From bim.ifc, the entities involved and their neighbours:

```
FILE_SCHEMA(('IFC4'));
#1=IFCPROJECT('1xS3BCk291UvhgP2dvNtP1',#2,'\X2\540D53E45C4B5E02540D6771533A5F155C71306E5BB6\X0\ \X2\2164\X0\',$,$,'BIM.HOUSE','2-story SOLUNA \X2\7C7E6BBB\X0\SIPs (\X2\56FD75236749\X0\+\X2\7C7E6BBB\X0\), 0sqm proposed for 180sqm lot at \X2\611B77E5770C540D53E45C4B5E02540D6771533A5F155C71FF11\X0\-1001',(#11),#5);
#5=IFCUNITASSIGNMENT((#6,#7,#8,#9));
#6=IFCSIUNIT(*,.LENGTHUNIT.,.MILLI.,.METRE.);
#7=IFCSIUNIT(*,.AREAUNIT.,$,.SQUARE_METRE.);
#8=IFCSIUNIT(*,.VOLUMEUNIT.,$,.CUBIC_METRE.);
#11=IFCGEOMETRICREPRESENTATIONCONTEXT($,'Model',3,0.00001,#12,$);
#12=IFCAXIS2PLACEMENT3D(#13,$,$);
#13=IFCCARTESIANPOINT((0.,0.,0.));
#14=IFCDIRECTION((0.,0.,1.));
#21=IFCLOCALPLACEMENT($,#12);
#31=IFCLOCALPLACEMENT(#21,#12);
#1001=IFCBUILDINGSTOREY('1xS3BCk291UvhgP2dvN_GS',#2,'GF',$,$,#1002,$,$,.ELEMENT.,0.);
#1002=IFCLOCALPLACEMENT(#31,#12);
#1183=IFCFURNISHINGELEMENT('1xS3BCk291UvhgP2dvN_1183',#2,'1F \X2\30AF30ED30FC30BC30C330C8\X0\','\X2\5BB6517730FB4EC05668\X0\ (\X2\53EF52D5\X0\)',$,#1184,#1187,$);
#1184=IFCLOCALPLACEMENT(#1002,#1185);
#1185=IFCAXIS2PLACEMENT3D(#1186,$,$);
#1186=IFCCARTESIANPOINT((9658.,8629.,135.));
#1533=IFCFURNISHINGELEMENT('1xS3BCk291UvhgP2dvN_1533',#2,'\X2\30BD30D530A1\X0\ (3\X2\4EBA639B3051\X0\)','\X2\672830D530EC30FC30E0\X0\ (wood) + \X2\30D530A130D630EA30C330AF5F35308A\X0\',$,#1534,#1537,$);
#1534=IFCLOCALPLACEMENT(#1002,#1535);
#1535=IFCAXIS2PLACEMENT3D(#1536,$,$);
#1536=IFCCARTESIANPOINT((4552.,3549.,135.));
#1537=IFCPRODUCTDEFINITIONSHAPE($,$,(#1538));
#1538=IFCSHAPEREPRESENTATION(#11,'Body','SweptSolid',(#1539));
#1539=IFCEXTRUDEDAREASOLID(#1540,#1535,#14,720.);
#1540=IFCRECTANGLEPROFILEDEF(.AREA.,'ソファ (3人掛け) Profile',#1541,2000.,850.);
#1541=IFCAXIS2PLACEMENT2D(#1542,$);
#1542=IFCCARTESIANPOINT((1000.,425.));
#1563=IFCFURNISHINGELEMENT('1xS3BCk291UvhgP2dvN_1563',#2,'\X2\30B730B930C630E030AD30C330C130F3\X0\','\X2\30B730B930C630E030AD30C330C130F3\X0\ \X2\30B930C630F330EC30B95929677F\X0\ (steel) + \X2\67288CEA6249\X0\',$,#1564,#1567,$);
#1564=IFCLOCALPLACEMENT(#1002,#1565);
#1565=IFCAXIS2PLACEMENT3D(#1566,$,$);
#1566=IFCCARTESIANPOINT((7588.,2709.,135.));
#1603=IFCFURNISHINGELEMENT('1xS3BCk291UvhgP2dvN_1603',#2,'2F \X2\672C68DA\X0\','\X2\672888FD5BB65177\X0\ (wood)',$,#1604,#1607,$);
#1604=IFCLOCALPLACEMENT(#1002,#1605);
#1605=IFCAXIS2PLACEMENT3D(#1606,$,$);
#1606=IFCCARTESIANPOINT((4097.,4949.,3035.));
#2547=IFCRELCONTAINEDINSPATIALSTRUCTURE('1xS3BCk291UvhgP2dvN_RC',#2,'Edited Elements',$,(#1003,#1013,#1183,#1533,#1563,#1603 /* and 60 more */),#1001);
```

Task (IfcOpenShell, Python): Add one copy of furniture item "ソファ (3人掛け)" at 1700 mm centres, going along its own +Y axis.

```python
import ifcopenshell
import ifcopenshell.api.geometry
import ifcopenshell.api.root
import ifcopenshell.util.element
import ifcopenshell.util.placement

model = ifcopenshell.open("bim.ifc")


def reuse_history(source, copy):
    """copy_class also copies each property set's owner history, people and application; keep the originals."""
    for rel in copy.IsDefinedBy:
        if rel.is_a("IfcRelDefinesByProperties") and (history := rel.RelatingPropertyDefinition.OwnerHistory):
            rel.RelatingPropertyDefinition.OwnerHistory = source.OwnerHistory
            ifcopenshell.util.element.remove_deep2(model, history)


source = model.by_guid("1xS3BCk291UvhgP2dvN_1533")
base = ifcopenshell.util.placement.get_local_placement(source.ObjectPlacement)
step = base[:3, 1] * 1700.0

for i in range(1, 2):
    copy = ifcopenshell.api.root.copy_class(model, product=source)
    copy.Representation = ifcopenshell.util.element.copy_deep(
        model, source.Representation, exclude=["IfcGeometricRepresentationContext", "IfcRepresentationMap"]
    )
    reuse_history(source, copy)
    matrix = base.copy()
    matrix[:3, 3] += i * step
    print("added at", matrix[:3, 3].round(3) + 0.0)
    ifcopenshell.api.geometry.edit_object_placement(model, product=copy, matrix=matrix, is_si=False)

model.write("bim_v2.ifc")
```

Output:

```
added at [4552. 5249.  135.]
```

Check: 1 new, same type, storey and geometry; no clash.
